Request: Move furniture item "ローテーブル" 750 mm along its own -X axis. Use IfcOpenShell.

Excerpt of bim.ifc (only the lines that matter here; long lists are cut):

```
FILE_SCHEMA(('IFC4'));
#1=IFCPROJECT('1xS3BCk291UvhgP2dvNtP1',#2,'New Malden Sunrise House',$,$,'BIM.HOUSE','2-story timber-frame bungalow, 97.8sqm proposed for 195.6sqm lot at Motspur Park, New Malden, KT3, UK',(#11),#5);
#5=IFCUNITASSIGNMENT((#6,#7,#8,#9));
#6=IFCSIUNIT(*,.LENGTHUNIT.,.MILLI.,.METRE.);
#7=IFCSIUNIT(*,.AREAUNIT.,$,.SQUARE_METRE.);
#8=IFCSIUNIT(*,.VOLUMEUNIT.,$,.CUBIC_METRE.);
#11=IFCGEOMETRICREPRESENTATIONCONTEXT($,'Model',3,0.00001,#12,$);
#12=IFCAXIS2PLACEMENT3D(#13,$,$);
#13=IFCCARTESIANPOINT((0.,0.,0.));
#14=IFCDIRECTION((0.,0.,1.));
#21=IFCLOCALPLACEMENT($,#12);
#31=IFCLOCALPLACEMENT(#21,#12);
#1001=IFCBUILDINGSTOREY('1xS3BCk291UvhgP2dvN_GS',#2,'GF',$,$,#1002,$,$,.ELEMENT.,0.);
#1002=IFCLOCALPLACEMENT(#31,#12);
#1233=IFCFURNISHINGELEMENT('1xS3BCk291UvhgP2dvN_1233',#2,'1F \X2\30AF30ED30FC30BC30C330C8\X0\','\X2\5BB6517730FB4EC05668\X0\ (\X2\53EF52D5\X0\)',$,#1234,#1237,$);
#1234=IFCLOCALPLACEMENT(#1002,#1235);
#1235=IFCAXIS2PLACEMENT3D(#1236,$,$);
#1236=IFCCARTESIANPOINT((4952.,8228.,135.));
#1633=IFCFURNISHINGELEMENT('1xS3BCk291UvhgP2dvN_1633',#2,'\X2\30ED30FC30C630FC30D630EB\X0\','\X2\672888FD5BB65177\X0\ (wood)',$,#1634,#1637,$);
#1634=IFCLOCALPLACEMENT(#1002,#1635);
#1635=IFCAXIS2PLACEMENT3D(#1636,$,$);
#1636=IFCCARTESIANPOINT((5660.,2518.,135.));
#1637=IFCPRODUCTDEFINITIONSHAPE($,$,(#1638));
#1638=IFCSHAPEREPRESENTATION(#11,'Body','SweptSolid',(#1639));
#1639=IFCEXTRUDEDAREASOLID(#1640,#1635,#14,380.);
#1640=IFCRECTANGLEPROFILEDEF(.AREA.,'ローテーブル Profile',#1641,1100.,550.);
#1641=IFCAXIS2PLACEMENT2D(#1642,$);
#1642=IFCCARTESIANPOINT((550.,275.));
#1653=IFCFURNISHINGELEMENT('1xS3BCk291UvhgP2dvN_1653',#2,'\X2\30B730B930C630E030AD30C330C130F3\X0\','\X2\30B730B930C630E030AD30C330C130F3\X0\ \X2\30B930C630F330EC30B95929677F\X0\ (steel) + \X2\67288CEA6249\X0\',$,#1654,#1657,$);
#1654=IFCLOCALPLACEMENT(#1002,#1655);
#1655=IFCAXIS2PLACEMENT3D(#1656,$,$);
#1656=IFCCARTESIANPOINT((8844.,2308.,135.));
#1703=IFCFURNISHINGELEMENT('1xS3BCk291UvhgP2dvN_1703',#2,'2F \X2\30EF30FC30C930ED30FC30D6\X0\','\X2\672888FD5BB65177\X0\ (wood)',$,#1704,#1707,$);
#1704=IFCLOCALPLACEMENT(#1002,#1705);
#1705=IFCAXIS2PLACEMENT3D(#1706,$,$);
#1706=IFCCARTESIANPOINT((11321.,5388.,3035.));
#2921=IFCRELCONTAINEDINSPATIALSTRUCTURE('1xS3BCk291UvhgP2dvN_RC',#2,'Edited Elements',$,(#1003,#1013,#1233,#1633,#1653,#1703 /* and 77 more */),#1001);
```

```python
import ifcopenshell
import ifcopenshell.api.geometry
import ifcopenshell.util.placement
import ifcopenshell.util.unit

model = ifcopenshell.open("bim.ifc")
unit_scale = ifcopenshell.util.unit.calculate_unit_scale(model)

item = model.by_guid("1xS3BCk291UvhgP2dvN_1633")
matrix = ifcopenshell.util.placement.get_local_placement(item.ObjectPlacement)
matrix[:3, 3] -= matrix[:3, 0] * 0.75 / unit_scale
ifcopenshell.api.geometry.edit_object_placement(model, product=item, matrix=matrix, is_si=False)

print(ifcopenshell.util.placement.get_local_placement(item.ObjectPlacement).round(3) + 0.0)

model.write("bim_v2.ifc")
```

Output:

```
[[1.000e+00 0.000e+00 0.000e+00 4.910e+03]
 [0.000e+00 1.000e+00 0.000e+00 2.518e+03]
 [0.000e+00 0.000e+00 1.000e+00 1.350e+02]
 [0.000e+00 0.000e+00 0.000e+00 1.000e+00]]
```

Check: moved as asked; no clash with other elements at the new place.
